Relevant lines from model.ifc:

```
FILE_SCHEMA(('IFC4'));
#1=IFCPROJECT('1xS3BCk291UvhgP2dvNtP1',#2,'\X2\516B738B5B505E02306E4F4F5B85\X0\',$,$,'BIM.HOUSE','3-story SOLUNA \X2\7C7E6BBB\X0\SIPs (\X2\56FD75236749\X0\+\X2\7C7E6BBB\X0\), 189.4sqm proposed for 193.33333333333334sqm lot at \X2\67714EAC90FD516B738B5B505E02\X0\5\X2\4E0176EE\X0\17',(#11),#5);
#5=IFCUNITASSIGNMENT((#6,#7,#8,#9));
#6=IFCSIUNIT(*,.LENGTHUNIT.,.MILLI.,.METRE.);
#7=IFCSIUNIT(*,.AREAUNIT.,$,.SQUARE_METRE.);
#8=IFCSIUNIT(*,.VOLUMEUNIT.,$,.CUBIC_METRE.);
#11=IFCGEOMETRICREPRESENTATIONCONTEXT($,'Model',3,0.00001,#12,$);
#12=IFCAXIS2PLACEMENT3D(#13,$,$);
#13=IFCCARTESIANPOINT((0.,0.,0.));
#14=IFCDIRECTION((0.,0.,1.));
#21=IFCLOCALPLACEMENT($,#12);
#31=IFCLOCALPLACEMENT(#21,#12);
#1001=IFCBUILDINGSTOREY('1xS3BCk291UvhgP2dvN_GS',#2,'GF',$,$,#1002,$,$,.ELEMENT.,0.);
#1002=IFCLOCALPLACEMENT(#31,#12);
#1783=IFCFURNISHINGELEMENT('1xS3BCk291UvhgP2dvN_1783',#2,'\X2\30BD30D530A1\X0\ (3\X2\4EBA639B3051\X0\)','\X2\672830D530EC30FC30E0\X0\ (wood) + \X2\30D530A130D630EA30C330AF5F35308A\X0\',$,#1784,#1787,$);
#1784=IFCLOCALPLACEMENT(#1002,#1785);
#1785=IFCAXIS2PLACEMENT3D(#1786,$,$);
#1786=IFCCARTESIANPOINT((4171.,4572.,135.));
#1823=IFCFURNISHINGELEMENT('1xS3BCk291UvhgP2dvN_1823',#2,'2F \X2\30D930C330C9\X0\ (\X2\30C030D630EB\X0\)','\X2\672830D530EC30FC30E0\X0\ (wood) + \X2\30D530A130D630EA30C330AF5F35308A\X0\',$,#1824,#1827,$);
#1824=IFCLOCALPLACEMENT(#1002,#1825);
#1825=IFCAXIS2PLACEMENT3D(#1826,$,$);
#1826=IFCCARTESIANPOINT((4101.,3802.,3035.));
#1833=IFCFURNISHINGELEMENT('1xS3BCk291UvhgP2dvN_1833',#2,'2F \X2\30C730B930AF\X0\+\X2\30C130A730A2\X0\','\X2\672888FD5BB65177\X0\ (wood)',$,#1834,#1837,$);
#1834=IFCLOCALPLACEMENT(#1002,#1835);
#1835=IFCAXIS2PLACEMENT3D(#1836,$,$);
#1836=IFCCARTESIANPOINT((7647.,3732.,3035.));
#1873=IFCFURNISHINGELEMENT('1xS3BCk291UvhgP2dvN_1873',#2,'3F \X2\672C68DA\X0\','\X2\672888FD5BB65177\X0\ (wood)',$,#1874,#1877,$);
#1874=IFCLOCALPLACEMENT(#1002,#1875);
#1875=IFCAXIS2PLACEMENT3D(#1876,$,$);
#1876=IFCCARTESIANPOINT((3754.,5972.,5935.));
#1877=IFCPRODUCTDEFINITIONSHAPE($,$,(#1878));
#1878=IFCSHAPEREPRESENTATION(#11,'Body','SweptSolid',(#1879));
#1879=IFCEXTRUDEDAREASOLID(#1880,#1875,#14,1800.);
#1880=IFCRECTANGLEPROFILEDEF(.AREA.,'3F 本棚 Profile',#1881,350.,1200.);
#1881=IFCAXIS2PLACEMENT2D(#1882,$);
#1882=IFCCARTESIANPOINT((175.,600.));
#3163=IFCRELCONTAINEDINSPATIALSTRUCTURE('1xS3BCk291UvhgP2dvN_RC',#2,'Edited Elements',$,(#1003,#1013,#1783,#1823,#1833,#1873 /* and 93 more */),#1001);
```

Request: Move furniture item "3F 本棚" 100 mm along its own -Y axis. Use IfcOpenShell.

```python
import ifcopenshell
import ifcopenshell.api.geometry
import ifcopenshell.util.placement
import ifcopenshell.util.unit

model = ifcopenshell.open("model.ifc")
unit_scale = ifcopenshell.util.unit.calculate_unit_scale(model)

item = model.by_guid("1xS3BCk291UvhgP2dvN_1873")
matrix = ifcopenshell.util.placement.get_local_placement(item.ObjectPlacement)
matrix[:3, 3] -= matrix[:3, 1] * 0.1 / unit_scale
ifcopenshell.api.geometry.edit_object_placement(model, product=item, matrix=matrix, is_si=False)

print(ifcopenshell.util.placement.get_local_placement(item.ObjectPlacement).round(3) + 0.0)

model.write("model_v2.ifc")
```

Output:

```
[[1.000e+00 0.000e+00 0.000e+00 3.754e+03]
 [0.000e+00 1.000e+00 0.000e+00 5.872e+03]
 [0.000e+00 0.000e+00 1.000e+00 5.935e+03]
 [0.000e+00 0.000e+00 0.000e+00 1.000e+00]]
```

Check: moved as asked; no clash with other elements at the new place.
